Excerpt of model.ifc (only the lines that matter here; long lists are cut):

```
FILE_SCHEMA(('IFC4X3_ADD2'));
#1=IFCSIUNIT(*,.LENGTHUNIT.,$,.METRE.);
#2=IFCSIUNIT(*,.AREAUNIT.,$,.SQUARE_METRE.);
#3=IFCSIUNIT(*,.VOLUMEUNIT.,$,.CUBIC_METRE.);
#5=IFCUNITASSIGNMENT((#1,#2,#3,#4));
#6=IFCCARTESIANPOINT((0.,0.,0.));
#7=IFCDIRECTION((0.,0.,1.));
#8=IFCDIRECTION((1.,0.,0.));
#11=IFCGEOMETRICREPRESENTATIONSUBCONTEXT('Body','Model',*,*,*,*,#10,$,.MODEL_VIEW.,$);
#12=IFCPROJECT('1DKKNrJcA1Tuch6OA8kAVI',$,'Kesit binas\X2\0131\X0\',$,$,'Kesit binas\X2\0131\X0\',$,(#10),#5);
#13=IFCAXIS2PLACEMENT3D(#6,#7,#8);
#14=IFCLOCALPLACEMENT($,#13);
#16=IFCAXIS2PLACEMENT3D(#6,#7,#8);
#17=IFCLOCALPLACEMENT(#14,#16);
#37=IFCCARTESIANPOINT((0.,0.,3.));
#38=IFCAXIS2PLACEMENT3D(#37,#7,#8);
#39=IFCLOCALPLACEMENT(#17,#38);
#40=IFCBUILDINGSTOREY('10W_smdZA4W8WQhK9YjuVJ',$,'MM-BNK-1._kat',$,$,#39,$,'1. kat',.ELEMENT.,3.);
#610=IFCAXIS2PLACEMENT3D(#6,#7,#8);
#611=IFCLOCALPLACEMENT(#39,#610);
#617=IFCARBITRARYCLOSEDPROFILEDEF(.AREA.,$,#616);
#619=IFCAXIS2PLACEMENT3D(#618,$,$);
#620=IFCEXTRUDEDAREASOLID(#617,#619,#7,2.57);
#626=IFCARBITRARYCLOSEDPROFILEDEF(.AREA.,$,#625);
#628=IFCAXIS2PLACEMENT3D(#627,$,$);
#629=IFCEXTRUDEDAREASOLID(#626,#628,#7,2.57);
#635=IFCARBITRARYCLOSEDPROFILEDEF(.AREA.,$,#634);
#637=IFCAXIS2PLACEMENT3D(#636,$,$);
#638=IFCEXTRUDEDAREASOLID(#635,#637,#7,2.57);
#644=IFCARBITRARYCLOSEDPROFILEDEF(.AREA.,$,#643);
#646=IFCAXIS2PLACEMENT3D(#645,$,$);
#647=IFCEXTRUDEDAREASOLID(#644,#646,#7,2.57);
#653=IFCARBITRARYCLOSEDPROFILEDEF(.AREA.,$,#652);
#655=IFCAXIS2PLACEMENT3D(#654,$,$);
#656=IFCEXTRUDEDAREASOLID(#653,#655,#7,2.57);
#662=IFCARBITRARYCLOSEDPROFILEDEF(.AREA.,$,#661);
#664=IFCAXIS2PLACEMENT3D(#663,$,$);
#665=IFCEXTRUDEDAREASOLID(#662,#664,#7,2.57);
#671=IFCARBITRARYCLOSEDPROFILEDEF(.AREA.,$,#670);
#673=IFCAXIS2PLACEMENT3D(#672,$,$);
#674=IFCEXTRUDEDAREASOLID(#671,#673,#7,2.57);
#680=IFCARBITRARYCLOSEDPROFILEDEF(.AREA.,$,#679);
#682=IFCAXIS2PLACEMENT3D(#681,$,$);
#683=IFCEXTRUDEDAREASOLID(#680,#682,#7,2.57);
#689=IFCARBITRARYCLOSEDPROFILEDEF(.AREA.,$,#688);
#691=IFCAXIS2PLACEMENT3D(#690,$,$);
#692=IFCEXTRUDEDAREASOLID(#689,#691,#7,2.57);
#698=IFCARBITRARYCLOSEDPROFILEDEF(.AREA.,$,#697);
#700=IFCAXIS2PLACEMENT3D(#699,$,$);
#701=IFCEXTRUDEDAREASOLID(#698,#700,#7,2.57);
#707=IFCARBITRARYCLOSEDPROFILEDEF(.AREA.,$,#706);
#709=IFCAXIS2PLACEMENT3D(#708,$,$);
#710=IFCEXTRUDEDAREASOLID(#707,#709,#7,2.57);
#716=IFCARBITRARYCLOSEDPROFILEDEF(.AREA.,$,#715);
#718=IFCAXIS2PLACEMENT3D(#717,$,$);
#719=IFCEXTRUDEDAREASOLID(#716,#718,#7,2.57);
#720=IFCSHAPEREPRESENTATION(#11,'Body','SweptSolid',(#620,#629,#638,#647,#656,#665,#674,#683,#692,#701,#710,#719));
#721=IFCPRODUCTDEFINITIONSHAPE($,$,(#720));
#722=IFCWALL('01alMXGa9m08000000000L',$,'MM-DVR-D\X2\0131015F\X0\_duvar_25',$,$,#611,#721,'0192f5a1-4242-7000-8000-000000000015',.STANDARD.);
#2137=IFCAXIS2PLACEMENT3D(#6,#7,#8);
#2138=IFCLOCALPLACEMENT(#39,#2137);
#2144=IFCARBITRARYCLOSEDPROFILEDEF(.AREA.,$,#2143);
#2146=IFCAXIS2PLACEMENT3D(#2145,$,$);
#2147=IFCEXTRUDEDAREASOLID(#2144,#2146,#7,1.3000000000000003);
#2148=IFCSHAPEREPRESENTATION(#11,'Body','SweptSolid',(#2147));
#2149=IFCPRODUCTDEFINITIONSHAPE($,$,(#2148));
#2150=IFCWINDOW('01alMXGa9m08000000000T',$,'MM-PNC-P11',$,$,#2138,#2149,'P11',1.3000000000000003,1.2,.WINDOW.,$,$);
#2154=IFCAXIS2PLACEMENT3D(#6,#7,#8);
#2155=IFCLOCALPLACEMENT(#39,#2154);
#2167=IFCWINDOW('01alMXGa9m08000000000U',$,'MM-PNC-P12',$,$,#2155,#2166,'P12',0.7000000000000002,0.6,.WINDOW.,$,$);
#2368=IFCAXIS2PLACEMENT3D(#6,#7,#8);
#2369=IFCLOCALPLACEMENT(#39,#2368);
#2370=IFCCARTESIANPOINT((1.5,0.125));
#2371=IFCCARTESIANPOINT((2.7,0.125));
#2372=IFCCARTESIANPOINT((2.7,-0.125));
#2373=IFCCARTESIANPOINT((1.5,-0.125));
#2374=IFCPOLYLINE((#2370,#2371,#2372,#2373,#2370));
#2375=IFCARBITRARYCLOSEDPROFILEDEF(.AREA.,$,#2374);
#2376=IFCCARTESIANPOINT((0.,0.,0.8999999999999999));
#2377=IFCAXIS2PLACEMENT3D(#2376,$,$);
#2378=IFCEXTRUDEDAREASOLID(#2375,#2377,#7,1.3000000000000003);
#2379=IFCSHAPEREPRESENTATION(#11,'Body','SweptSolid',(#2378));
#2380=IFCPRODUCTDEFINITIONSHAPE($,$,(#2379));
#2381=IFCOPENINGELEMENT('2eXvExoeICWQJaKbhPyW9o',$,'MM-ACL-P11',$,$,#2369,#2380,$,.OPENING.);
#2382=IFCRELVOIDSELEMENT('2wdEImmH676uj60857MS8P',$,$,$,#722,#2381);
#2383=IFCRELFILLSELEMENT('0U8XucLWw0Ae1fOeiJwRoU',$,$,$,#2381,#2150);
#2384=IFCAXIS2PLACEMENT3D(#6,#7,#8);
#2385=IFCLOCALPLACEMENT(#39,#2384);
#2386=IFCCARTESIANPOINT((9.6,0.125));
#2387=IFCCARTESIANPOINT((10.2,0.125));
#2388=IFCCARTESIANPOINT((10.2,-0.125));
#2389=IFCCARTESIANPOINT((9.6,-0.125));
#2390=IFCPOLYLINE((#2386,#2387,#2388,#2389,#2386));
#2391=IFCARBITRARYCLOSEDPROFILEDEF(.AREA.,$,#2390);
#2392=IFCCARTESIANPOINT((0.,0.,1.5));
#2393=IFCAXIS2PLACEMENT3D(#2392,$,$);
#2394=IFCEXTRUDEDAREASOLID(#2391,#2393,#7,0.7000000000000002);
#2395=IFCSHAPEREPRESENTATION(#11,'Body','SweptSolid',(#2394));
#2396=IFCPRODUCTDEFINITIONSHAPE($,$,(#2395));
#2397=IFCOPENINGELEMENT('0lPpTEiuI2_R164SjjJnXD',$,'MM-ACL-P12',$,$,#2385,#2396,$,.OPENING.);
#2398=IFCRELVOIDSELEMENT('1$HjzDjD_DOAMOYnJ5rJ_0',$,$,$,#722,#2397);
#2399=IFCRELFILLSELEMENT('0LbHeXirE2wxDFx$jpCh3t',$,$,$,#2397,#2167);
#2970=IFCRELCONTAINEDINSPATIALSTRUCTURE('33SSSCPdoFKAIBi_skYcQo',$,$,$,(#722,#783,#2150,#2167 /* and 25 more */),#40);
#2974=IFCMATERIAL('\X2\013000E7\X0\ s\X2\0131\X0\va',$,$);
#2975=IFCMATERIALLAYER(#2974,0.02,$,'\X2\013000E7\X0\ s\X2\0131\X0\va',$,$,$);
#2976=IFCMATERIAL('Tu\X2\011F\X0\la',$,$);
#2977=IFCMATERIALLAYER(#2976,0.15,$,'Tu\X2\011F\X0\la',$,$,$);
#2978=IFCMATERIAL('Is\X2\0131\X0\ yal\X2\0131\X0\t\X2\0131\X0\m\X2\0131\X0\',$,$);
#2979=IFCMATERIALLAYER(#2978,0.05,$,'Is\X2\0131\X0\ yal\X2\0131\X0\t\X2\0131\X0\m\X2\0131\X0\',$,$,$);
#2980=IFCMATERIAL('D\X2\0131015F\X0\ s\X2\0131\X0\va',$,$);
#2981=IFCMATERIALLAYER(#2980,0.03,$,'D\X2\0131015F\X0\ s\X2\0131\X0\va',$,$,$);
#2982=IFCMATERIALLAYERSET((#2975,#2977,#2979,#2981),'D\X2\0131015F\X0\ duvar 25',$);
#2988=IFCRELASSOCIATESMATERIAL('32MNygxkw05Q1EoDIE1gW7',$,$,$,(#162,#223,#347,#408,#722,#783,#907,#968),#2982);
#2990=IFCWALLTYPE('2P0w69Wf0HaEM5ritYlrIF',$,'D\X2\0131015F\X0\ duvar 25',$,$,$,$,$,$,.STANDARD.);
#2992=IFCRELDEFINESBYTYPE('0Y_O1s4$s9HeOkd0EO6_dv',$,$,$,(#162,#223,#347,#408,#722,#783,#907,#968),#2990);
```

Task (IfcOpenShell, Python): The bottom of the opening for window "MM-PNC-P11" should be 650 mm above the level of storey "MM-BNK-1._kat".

```python
import numpy as np
import ifcopenshell
import ifcopenshell.api.geometry
import ifcopenshell.geom
import ifcopenshell.util.element
import ifcopenshell.util.placement
import ifcopenshell.util.shape
import ifcopenshell.util.unit

model = ifcopenshell.open("model.ifc")
unit_scale = ifcopenshell.util.unit.calculate_unit_scale(model)

window = model.by_guid("01alMXGa9m08000000000T")
opening = window.FillsVoids[0].RelatingOpeningElement
storey = ifcopenshell.util.element.get_container(window, ifc_class="IfcBuildingStorey")
level = ifcopenshell.util.placement.get_local_placement(storey.ObjectPlacement)[2, 3]

# The opening's origin need not be at the sill, so measure its lowest point.
shape = ifcopenshell.geom.create_shape(ifcopenshell.geom.settings(), opening)
bottom = ifcopenshell.util.shape.get_shape_bottom_elevation(shape, shape.geometry) / unit_scale
dz = level + 0.65 / unit_scale - bottom

shift = np.array([0.0, 0.0, dz])
# The window is not placed relative to its opening, so move both.
for product in (opening, window):
    matrix = ifcopenshell.util.placement.get_local_placement(product.ObjectPlacement)
    matrix[:3, 3] += shift
    ifcopenshell.api.geometry.edit_object_placement(model, product=product, matrix=matrix, is_si=False)

print(f"moved by {dz * unit_scale:+.3f} m")

model.write("model_edited.ifc")
```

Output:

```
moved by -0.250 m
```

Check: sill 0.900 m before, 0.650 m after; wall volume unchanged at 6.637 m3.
